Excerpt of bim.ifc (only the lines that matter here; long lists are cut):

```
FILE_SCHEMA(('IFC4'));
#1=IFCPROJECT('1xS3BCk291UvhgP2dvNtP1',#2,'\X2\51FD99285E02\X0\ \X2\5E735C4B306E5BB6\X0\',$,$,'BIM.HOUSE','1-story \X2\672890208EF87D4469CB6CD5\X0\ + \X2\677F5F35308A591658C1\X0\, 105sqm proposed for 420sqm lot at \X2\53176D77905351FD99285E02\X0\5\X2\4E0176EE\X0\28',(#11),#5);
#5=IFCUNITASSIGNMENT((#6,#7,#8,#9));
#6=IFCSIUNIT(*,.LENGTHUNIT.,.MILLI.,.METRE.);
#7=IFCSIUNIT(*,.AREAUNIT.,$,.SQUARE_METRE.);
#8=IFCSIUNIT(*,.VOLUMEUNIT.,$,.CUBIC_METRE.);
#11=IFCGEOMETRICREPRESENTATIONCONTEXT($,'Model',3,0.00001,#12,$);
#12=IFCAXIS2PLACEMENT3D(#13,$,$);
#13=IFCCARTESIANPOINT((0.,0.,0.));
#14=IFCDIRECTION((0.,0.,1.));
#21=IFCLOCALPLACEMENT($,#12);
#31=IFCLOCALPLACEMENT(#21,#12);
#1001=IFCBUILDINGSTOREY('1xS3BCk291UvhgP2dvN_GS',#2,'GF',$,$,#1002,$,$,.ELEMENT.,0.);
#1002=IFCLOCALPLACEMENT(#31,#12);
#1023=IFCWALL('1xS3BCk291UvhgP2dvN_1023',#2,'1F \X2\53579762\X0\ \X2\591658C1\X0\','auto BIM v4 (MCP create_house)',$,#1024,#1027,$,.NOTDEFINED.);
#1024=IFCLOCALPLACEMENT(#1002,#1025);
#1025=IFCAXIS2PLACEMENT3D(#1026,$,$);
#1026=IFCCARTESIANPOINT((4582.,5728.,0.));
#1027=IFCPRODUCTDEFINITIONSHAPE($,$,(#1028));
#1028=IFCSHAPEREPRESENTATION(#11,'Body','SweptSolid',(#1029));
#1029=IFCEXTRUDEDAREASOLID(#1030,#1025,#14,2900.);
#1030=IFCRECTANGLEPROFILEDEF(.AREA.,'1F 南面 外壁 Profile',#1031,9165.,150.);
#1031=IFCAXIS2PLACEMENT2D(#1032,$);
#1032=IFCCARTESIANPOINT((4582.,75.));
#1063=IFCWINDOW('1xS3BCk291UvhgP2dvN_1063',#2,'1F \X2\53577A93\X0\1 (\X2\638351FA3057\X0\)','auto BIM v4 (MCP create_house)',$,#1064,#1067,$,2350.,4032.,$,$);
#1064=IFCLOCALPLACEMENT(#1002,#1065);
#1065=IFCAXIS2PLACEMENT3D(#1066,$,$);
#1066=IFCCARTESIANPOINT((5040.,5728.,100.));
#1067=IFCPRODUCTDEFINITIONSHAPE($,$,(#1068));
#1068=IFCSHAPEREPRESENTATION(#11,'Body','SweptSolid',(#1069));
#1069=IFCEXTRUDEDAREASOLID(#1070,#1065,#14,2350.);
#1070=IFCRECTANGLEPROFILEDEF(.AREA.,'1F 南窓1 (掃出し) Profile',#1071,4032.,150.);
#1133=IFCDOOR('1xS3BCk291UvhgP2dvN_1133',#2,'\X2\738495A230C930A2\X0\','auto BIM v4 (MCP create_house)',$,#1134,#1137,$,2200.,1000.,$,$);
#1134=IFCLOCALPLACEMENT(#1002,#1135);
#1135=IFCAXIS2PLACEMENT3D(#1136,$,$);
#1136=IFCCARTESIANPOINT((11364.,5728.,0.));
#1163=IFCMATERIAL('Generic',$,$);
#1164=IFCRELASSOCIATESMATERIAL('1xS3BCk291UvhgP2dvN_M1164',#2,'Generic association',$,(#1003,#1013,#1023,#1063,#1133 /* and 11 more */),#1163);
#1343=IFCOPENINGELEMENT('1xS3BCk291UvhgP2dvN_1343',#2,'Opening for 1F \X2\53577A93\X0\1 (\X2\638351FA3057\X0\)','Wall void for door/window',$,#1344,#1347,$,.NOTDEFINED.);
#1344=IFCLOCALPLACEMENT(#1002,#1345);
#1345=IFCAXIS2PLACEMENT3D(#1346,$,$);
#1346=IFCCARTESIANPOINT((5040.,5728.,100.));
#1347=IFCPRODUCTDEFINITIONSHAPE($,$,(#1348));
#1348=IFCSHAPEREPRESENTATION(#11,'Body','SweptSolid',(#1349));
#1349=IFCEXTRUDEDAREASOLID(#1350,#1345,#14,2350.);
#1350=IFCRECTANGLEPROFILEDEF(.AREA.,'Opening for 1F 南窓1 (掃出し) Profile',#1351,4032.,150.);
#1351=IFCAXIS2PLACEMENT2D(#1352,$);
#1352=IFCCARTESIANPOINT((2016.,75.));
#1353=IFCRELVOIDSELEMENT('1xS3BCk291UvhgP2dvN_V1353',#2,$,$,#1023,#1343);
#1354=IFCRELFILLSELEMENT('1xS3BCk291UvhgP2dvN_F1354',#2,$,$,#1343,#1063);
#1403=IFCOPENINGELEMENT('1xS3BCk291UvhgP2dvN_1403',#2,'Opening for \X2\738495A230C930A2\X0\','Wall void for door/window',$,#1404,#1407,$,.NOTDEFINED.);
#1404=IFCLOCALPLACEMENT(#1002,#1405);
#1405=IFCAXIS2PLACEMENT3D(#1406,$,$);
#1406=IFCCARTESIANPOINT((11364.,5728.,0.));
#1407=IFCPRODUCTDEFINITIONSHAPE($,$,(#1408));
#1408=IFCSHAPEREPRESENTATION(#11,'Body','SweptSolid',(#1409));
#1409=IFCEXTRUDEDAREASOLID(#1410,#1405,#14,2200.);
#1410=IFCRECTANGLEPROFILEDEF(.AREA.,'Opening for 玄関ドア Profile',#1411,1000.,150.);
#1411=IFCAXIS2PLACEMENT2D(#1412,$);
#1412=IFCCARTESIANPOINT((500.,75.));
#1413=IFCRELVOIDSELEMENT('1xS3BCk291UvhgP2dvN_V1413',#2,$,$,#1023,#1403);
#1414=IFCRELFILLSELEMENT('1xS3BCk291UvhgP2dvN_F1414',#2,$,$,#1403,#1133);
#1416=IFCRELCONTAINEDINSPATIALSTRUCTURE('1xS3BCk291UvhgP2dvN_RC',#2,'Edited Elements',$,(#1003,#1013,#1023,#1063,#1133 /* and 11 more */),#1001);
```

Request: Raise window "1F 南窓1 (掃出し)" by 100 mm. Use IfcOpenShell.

```python
import numpy as np
import ifcopenshell
import ifcopenshell.api.geometry
import ifcopenshell.util.placement
import ifcopenshell.util.unit

model = ifcopenshell.open("bim.ifc")
unit_scale = ifcopenshell.util.unit.calculate_unit_scale(model)

window = model.by_guid("1xS3BCk291UvhgP2dvN_1063")
opening = window.FillsVoids[0].RelatingOpeningElement
dz = 100.0

shift = np.array([0.0, 0.0, dz])
# The window is not placed relative to its opening, so move both.
for product in (opening, window):
    matrix = ifcopenshell.util.placement.get_local_placement(product.ObjectPlacement)
    matrix[:3, 3] += shift
    ifcopenshell.api.geometry.edit_object_placement(model, product=product, matrix=matrix, is_si=False)

print(f"moved by {dz * unit_scale:+.3f} m")

model.write("bim_edited.ifc")
```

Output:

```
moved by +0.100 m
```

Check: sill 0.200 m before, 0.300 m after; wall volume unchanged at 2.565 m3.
